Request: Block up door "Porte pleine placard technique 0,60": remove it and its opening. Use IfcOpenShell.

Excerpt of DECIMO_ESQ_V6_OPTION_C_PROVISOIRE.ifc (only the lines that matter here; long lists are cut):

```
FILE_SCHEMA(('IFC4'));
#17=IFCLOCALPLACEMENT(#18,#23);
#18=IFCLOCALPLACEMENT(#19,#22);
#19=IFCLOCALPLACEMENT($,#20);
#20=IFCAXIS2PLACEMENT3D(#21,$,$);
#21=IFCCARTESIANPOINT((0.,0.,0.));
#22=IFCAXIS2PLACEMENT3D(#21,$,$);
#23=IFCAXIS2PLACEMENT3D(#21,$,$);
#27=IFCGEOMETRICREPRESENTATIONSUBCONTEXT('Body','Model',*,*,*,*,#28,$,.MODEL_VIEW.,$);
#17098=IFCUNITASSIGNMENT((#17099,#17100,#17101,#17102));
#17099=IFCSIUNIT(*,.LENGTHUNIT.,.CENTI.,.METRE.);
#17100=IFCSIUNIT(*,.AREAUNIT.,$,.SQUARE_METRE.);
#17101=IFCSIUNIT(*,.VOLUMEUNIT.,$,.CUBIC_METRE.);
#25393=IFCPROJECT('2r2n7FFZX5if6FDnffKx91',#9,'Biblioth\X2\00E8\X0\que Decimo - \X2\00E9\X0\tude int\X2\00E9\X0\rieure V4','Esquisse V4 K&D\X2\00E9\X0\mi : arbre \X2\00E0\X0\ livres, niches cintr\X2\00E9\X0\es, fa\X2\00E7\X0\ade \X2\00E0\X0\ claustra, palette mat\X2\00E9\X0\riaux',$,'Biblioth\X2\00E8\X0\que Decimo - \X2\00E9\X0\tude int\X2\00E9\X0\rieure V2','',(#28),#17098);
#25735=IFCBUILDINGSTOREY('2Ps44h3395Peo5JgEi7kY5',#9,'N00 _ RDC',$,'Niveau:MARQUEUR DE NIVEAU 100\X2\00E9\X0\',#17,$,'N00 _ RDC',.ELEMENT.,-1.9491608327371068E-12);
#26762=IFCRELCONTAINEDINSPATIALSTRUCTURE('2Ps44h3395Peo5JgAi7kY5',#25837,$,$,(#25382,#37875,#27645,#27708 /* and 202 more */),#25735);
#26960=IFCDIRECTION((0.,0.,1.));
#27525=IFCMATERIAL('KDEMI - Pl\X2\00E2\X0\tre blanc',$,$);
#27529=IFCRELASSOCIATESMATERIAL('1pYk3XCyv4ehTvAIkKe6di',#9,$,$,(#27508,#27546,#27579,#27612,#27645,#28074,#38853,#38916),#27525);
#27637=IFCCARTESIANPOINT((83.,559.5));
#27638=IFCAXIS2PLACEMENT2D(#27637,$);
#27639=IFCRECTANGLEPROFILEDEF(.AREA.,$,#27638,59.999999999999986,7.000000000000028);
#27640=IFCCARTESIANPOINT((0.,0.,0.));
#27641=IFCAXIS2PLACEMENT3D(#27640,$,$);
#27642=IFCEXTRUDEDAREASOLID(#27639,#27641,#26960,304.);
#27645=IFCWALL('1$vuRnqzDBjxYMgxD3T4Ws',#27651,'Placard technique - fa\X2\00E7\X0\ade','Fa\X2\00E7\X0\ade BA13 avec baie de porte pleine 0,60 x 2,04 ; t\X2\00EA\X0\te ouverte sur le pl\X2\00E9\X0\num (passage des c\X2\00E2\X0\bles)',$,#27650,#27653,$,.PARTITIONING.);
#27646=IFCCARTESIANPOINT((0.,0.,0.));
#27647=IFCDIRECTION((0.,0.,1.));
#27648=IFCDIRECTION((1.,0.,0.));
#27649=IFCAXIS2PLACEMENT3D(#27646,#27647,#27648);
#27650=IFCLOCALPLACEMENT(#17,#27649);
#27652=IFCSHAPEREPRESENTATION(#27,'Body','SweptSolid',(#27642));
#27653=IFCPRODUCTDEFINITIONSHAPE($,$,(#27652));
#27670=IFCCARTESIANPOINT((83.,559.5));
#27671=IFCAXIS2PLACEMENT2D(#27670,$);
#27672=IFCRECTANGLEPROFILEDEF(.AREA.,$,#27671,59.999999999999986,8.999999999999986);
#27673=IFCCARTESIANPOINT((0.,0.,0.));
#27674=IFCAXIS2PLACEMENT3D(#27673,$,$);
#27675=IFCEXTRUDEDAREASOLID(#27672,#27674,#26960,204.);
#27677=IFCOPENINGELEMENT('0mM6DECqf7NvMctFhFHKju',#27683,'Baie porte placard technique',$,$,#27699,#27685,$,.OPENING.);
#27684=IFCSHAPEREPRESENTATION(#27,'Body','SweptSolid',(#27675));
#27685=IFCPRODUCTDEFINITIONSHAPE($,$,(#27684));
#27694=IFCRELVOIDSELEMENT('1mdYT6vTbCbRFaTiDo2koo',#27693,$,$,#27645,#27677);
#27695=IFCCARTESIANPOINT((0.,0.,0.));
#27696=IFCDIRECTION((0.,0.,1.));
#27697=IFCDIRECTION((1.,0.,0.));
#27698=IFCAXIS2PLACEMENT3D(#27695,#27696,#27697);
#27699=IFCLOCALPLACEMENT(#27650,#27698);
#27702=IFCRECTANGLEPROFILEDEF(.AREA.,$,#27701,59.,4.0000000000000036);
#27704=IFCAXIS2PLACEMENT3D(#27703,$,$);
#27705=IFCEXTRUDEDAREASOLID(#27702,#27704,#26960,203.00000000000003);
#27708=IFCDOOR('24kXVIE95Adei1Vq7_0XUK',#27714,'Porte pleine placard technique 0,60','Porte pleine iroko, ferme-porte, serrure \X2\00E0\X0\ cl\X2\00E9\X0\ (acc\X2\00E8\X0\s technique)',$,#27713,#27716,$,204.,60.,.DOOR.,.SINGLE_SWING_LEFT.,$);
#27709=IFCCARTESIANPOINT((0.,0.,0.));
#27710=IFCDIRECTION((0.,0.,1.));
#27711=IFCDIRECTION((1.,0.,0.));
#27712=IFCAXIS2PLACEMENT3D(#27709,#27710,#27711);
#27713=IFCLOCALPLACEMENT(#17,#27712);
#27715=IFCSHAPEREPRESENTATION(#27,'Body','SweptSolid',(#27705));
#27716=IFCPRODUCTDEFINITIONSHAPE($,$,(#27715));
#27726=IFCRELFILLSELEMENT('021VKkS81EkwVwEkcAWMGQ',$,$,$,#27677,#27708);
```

```python
import ifcopenshell
import ifcopenshell.api.feature
import ifcopenshell.api.root
import ifcopenshell.geom
import ifcopenshell.util.shape

model = ifcopenshell.open("DECIMO_ESQ_V6_OPTION_C_PROVISOIRE.ifc")
settings = ifcopenshell.geom.settings()


def volume(element):
    """Net volume in cubic metres, openings subtracted."""
    shape = ifcopenshell.geom.create_shape(settings, element)
    return ifcopenshell.util.shape.get_volume(shape.geometry)


door = model.by_guid("24kXVIE95Adei1Vq7_0XUK")
opening = door.FillsVoids[0].RelatingOpeningElement
wall = opening.VoidsElements[0].RelatingBuildingElement
before = volume(wall)

ifcopenshell.api.root.remove_product(model, product=door)
ifcopenshell.api.feature.remove_feature(model, feature=opening)

after = volume(wall)

print(f"wall volume {before:.3f} -> {after:.3f} m3")

model.write("DECIMO_ESQ_V6_OPTION_C_PROVISOIRE_v2.ifc")
```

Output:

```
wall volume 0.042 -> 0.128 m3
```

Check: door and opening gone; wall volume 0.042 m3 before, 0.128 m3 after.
